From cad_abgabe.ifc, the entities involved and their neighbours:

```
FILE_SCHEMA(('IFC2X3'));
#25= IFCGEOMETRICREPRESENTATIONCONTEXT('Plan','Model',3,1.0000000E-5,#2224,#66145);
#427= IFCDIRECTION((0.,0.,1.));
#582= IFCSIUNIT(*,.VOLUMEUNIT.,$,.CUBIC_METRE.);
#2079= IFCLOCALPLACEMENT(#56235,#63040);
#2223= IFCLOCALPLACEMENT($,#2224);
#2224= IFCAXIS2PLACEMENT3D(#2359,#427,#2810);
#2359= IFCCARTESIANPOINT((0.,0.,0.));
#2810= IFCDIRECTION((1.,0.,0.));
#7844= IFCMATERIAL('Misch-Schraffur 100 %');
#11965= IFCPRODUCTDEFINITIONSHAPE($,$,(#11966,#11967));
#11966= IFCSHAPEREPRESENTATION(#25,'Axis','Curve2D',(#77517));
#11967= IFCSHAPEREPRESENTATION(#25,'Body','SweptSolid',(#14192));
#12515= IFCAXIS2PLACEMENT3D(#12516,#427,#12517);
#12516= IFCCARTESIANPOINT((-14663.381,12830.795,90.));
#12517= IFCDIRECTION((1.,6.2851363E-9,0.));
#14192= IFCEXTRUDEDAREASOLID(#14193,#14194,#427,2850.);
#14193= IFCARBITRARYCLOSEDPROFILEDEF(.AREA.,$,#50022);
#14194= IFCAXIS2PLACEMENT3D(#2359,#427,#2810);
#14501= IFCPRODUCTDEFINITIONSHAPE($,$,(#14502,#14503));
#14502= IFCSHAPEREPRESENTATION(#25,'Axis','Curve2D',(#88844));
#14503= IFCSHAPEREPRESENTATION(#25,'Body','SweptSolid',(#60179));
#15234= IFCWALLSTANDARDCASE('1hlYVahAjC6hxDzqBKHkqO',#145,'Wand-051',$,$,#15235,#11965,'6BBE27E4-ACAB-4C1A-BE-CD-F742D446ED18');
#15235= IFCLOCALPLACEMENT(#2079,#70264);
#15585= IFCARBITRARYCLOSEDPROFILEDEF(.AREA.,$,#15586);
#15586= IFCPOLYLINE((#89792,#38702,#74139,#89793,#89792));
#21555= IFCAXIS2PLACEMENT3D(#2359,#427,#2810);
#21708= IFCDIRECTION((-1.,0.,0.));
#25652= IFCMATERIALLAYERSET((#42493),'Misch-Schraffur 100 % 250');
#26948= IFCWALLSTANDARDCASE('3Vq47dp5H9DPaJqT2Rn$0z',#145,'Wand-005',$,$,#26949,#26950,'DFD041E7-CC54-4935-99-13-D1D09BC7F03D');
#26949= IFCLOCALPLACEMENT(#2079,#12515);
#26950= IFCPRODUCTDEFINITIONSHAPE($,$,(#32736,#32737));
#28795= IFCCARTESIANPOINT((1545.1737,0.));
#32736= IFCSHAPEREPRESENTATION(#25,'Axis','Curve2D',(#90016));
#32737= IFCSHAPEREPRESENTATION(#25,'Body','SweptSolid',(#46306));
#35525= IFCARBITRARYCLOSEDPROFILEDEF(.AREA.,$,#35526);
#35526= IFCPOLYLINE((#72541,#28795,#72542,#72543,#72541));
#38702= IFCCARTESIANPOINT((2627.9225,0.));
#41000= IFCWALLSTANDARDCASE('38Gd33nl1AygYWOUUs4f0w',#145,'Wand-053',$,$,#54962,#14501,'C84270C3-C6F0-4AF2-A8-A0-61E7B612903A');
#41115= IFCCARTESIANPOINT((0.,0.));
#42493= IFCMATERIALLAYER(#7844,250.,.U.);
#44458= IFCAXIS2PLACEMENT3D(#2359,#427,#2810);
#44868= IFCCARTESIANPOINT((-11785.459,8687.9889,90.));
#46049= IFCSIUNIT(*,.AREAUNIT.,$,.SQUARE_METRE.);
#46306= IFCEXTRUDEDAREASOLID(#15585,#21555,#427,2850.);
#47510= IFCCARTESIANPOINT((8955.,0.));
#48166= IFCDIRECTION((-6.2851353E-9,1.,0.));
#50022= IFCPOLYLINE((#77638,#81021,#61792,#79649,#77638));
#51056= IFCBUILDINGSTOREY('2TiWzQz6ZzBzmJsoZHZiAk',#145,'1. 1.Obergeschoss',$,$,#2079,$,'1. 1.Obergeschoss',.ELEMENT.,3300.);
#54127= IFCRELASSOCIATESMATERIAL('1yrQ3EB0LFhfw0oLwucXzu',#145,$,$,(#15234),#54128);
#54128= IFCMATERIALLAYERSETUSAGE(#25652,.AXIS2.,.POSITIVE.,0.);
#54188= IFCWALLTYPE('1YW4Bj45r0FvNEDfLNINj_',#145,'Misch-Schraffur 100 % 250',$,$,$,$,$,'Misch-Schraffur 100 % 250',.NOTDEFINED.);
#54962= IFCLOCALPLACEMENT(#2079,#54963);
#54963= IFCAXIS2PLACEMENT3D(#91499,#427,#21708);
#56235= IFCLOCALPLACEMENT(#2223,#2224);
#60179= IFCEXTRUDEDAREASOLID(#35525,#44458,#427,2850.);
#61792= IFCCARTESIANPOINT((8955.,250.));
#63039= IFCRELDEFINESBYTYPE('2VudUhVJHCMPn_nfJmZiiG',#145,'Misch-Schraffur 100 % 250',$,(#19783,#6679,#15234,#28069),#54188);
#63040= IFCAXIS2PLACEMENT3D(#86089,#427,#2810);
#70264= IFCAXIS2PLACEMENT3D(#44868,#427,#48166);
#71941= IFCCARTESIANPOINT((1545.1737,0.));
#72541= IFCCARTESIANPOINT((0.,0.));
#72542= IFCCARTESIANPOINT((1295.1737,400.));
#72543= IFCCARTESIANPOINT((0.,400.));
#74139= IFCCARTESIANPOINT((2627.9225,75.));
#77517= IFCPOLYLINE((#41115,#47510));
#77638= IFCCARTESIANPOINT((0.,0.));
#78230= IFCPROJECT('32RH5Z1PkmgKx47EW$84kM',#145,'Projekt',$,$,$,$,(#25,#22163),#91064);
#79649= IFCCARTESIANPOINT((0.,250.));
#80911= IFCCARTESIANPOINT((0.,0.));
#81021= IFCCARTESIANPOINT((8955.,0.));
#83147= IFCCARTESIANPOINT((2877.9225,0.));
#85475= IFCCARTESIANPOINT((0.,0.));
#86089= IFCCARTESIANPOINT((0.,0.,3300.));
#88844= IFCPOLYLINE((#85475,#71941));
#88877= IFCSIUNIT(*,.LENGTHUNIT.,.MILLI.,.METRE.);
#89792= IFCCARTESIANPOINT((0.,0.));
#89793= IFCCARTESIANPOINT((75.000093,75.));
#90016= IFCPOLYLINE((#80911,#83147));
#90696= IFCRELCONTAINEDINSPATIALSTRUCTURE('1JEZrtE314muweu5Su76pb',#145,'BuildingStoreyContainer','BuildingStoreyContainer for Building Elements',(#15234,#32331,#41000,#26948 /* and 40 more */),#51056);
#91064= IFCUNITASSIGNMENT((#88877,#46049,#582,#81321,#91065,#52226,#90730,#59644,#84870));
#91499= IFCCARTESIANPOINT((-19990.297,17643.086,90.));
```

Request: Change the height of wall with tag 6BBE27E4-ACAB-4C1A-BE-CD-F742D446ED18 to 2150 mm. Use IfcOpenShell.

```python
import ifcopenshell
import ifcopenshell.geom
import ifcopenshell.util.shape
import ifcopenshell.util.unit

model = ifcopenshell.open("cad_abgabe.ifc")
unit_scale = ifcopenshell.util.unit.calculate_unit_scale(model)
settings = ifcopenshell.geom.settings()


def volume(element):
    """Net volume in cubic metres, openings subtracted."""
    shape = ifcopenshell.geom.create_shape(settings, element)
    return ifcopenshell.util.shape.get_volume(shape.geometry)


wall = model.by_guid("1hlYVahAjC6hxDzqBKHkqO")
before = volume(wall)

body = next(r for r in wall.Representation.Representations if r.RepresentationIdentifier == "Body")
solid = body.Items[0]
old_height = solid.Depth
solid.Depth = 2.15 / unit_scale
after = volume(wall)

print(f"height {old_height:g} -> {solid.Depth:g}, volume {before:.3f} -> {after:.3f} m3")

model.write("cad_abgabe_updated.ifc")
```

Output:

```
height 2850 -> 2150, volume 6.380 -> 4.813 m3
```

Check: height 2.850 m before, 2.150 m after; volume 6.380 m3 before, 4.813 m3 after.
